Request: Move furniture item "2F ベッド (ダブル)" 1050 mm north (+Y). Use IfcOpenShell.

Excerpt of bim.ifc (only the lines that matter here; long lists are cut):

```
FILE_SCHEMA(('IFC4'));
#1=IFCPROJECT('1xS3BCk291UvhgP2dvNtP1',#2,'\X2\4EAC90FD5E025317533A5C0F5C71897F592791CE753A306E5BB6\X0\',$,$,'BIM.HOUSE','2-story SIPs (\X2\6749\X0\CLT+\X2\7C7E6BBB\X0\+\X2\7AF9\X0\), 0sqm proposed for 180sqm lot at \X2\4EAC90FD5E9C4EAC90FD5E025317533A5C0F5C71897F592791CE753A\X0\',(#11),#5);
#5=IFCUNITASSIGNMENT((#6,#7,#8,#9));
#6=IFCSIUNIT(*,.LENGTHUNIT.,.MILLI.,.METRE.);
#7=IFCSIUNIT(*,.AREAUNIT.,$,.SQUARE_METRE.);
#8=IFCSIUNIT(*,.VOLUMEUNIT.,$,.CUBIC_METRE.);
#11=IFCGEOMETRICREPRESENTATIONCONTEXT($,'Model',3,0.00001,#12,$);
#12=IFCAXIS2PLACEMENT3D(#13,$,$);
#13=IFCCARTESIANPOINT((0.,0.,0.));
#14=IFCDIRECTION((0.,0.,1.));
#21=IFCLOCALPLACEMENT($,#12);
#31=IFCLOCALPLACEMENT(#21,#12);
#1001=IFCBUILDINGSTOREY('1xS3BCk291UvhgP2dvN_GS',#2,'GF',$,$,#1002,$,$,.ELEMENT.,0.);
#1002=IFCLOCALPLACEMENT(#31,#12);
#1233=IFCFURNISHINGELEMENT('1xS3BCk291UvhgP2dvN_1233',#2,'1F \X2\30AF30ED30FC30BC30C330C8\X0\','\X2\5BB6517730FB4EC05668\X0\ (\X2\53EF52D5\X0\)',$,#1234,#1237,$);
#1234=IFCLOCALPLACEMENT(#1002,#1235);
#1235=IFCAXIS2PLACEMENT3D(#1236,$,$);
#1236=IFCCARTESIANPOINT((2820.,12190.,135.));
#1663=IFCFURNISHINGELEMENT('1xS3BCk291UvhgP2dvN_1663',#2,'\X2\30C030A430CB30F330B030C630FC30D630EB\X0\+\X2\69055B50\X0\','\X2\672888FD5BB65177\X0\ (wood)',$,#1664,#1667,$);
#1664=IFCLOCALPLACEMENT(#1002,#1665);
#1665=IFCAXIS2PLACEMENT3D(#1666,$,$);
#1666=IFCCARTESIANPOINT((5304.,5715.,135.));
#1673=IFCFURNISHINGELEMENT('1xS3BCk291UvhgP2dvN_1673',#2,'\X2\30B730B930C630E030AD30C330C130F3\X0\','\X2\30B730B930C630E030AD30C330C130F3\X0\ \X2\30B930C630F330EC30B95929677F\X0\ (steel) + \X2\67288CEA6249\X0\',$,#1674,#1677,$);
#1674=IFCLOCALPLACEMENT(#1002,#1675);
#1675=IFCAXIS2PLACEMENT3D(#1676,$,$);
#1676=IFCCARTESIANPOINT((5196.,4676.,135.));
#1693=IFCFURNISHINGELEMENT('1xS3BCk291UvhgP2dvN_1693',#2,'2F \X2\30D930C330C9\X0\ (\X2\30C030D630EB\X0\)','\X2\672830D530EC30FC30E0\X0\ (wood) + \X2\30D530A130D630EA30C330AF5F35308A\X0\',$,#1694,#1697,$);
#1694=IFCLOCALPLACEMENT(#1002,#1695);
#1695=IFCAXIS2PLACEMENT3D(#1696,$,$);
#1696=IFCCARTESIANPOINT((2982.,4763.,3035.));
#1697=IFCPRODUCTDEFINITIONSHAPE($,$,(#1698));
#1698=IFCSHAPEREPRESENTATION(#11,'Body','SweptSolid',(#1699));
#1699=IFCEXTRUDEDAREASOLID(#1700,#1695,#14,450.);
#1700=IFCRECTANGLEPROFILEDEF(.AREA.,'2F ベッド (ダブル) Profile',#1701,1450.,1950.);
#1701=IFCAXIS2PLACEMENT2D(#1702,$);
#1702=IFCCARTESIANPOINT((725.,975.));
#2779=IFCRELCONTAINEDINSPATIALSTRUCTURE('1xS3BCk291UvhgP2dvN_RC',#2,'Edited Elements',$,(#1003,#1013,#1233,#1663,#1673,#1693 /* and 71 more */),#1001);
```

```python
import ifcopenshell
import ifcopenshell.api.geometry
import ifcopenshell.util.placement
import ifcopenshell.util.unit

model = ifcopenshell.open("bim.ifc")
unit_scale = ifcopenshell.util.unit.calculate_unit_scale(model)

item = model.by_guid("1xS3BCk291UvhgP2dvN_1693")
matrix = ifcopenshell.util.placement.get_local_placement(item.ObjectPlacement)
matrix[1, 3] += 1.05 / unit_scale
ifcopenshell.api.geometry.edit_object_placement(model, product=item, matrix=matrix, is_si=False)

print(ifcopenshell.util.placement.get_local_placement(item.ObjectPlacement).round(3) + 0.0)

model.write("bim_v2.ifc")
```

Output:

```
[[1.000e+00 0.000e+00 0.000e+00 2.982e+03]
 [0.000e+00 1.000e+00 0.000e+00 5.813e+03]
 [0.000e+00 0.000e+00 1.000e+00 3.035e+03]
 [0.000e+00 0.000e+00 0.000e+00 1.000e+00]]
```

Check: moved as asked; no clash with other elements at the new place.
